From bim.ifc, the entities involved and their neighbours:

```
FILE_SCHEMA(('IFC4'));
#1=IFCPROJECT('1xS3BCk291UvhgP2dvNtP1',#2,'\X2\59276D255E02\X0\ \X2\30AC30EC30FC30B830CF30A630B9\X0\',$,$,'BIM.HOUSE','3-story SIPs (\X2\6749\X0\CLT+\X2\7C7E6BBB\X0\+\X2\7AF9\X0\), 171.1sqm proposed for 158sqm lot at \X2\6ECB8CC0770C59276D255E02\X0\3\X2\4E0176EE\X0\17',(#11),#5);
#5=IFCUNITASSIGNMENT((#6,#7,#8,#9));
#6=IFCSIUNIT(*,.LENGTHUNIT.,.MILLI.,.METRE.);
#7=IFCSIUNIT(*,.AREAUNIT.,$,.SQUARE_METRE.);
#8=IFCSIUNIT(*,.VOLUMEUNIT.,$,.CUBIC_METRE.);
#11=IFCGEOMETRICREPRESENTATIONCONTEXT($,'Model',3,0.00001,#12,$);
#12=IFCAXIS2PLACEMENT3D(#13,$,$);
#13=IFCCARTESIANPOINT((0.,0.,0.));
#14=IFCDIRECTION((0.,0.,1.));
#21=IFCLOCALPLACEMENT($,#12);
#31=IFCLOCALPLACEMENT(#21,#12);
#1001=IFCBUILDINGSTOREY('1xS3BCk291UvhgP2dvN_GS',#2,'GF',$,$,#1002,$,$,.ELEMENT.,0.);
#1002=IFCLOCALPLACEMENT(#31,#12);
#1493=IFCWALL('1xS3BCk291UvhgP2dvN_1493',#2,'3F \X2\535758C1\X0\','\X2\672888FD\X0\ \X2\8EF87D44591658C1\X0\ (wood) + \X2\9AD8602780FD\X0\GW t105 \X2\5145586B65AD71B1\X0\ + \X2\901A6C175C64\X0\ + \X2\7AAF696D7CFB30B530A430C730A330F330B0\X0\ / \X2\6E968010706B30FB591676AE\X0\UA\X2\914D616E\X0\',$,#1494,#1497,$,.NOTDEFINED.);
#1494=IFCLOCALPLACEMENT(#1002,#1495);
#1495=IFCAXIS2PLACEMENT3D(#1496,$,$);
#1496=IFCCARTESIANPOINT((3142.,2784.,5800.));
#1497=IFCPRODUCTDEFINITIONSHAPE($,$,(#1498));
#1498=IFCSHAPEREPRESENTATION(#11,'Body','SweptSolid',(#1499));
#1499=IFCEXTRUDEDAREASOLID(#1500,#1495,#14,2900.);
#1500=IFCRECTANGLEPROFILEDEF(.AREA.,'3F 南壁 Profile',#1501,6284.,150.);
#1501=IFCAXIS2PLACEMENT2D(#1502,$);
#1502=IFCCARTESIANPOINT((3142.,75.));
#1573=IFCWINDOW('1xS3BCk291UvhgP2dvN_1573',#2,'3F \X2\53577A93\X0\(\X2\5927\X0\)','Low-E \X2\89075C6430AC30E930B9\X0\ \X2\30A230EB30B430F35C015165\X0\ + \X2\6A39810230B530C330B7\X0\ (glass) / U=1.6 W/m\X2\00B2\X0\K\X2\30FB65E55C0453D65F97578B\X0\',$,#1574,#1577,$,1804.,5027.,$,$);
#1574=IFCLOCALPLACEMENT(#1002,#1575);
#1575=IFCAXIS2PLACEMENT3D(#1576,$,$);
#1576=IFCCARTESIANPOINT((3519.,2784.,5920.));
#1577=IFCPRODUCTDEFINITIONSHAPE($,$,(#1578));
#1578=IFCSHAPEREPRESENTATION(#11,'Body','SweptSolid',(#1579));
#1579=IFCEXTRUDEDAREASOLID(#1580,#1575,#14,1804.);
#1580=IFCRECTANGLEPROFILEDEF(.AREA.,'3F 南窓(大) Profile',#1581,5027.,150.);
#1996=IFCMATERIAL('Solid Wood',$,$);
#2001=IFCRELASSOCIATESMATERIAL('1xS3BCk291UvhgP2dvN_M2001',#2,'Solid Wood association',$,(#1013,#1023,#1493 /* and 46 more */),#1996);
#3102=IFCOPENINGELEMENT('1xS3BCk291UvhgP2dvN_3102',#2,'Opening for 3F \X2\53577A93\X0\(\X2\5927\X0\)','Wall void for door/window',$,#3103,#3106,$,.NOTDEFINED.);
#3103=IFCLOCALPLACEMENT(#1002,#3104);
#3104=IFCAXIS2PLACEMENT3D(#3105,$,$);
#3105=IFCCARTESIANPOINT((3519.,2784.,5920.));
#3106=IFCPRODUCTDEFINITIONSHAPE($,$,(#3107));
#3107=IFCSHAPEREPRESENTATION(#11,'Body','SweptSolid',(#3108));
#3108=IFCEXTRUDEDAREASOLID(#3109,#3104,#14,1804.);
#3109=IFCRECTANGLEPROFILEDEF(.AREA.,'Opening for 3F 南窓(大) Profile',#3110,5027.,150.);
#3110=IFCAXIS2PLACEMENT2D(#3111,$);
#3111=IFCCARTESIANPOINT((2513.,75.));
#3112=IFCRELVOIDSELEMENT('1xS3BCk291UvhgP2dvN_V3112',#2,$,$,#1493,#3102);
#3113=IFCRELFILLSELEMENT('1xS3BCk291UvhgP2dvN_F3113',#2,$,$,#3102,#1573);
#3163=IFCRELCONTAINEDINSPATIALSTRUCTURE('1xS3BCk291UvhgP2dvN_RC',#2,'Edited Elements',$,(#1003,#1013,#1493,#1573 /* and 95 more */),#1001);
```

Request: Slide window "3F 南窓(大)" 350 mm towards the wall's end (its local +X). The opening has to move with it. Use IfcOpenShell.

```python
import ifcopenshell
import ifcopenshell.api.geometry
import ifcopenshell.util.placement
import ifcopenshell.util.unit

model = ifcopenshell.open("bim.ifc")
unit_scale = ifcopenshell.util.unit.calculate_unit_scale(model)

window = model.by_guid("1xS3BCk291UvhgP2dvN_1573")
opening = window.FillsVoids[0].RelatingOpeningElement
wall = opening.VoidsElements[0].RelatingBuildingElement

wall_matrix = ifcopenshell.util.placement.get_local_placement(wall.ObjectPlacement)
shift = wall_matrix[:3, 0] * 0.35 / unit_scale
before = ifcopenshell.util.placement.get_local_placement(window.ObjectPlacement)[:3, 3].copy()

# The window is not placed relative to its opening, so move both.
for product in (opening, window):
    matrix = ifcopenshell.util.placement.get_local_placement(product.ObjectPlacement)
    matrix[:3, 3] += shift
    ifcopenshell.api.geometry.edit_object_placement(model, product=product, matrix=matrix, is_si=False)

after = ifcopenshell.util.placement.get_local_placement(window.ObjectPlacement)[:3, 3]
print("window moved by", (after - before).round(3) + 0.0)

model.write("bim_updated.ifc")
```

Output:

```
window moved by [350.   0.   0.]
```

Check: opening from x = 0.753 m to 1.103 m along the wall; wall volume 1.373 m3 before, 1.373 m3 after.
